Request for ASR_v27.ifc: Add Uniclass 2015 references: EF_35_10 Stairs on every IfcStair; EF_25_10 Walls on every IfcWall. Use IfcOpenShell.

First a look at what the model holds.

```python
import ifcopenshell

model = ifcopenshell.open("ASR_v27.ifc")
print(model.schema)
print("classifications:", [c.Name for c in model.by_type("IfcClassification")])
for ifc_class in ("IfcDoor", "IfcRoof", "IfcStair", "IfcWall", "IfcWindow"):
    print(ifc_class, len(model.by_type(ifc_class)))
```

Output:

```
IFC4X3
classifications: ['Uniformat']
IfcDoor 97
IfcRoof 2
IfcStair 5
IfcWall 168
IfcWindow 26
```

```python
import ifcopenshell
import ifcopenshell.api.classification

model = ifcopenshell.open("ASR_v27.ifc")

system = ifcopenshell.api.classification.add_classification(model, classification="Uniclass 2015")

codes = {
    "IfcStair": ("EF_35_10", "Stairs"),
    "IfcWall": ("EF_25_10", "Walls"),
}
for ifc_class, (code, name) in codes.items():
    products = model.by_type(ifc_class)
    ifcopenshell.api.classification.add_reference(
        model, products=products, classification=system, identification=code, name=name
    )
    print(code, len(products))

model.write("ASR_v27_updated.ifc")
```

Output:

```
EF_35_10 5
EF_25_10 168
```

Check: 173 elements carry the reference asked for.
